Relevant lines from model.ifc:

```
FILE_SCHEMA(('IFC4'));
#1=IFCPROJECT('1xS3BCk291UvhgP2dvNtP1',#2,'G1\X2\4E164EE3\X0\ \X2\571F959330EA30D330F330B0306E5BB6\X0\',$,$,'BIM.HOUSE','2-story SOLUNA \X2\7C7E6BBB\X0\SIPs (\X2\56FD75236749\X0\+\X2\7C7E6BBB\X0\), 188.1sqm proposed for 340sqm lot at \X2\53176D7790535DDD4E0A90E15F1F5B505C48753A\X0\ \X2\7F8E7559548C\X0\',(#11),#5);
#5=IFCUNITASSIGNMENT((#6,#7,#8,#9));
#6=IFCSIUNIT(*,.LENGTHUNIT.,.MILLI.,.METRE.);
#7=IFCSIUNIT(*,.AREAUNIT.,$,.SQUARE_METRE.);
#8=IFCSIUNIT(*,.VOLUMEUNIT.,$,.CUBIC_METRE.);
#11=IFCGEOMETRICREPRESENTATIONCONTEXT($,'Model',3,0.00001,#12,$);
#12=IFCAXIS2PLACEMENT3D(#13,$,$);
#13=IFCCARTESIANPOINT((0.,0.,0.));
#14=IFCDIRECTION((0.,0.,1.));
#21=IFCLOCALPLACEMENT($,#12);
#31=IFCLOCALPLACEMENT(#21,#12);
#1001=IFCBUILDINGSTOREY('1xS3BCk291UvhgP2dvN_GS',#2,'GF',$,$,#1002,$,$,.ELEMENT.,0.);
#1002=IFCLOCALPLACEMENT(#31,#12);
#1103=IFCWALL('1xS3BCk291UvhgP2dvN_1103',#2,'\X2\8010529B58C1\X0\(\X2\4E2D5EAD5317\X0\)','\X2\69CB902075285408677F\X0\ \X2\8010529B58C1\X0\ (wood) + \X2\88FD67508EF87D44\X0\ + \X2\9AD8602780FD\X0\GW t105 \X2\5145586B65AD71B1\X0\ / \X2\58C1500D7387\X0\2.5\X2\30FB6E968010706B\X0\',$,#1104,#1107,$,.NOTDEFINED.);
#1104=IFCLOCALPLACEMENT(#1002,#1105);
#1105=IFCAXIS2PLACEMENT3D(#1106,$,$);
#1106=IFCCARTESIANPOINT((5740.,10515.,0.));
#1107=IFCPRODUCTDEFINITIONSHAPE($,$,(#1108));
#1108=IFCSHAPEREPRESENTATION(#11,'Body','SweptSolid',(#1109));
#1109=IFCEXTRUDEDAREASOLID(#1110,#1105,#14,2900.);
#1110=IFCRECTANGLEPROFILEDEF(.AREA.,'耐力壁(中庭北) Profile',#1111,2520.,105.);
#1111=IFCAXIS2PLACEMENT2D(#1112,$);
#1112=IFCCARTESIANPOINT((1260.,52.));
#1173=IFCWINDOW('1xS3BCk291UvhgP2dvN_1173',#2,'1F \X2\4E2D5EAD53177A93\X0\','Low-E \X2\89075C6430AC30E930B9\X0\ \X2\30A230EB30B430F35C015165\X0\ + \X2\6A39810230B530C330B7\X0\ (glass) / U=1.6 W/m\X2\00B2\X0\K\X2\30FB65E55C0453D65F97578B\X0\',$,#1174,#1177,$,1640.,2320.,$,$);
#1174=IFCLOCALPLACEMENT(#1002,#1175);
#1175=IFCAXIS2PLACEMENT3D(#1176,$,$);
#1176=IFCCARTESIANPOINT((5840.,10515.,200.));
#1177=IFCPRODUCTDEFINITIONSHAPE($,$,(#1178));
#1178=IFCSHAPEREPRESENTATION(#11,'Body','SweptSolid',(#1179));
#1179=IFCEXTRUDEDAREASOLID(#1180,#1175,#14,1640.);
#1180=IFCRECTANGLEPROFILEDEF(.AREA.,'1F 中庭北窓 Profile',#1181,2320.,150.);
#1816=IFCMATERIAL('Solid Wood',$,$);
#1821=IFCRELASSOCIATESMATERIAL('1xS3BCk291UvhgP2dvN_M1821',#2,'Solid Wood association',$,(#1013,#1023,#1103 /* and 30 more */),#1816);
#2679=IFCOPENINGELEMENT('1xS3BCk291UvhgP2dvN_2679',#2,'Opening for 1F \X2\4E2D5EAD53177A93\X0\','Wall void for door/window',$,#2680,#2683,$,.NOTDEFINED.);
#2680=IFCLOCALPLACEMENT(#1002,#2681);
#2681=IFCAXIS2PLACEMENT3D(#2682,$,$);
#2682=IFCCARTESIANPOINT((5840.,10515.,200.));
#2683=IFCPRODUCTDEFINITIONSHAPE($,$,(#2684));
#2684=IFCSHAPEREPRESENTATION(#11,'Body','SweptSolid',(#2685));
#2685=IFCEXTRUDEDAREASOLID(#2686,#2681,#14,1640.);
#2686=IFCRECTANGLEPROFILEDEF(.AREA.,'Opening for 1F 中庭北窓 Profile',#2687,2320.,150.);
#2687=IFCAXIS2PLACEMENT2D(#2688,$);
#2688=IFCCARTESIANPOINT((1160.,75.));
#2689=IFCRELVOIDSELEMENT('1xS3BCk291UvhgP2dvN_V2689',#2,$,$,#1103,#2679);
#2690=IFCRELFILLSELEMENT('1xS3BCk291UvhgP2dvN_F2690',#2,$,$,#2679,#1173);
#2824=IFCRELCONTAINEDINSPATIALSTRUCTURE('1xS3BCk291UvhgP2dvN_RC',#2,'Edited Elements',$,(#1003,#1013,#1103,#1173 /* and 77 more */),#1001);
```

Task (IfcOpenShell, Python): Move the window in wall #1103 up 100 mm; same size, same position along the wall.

```python
import numpy as np
import ifcopenshell
import ifcopenshell.api.geometry
import ifcopenshell.util.placement
import ifcopenshell.util.unit

model = ifcopenshell.open("model.ifc")
unit_scale = ifcopenshell.util.unit.calculate_unit_scale(model)

window = model.by_id(1173)
opening = window.FillsVoids[0].RelatingOpeningElement
dz = 0.1 / unit_scale

shift = np.array([0.0, 0.0, dz])
# The window is not placed relative to its opening, so move both.
for product in (opening, window):
    matrix = ifcopenshell.util.placement.get_local_placement(product.ObjectPlacement)
    matrix[:3, 3] += shift
    ifcopenshell.api.geometry.edit_object_placement(model, product=product, matrix=matrix, is_si=False)

print(f"moved by {dz * unit_scale:+.3f} m")

model.write("model_updated.ifc")
```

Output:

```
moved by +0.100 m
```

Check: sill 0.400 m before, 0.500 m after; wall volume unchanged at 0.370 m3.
